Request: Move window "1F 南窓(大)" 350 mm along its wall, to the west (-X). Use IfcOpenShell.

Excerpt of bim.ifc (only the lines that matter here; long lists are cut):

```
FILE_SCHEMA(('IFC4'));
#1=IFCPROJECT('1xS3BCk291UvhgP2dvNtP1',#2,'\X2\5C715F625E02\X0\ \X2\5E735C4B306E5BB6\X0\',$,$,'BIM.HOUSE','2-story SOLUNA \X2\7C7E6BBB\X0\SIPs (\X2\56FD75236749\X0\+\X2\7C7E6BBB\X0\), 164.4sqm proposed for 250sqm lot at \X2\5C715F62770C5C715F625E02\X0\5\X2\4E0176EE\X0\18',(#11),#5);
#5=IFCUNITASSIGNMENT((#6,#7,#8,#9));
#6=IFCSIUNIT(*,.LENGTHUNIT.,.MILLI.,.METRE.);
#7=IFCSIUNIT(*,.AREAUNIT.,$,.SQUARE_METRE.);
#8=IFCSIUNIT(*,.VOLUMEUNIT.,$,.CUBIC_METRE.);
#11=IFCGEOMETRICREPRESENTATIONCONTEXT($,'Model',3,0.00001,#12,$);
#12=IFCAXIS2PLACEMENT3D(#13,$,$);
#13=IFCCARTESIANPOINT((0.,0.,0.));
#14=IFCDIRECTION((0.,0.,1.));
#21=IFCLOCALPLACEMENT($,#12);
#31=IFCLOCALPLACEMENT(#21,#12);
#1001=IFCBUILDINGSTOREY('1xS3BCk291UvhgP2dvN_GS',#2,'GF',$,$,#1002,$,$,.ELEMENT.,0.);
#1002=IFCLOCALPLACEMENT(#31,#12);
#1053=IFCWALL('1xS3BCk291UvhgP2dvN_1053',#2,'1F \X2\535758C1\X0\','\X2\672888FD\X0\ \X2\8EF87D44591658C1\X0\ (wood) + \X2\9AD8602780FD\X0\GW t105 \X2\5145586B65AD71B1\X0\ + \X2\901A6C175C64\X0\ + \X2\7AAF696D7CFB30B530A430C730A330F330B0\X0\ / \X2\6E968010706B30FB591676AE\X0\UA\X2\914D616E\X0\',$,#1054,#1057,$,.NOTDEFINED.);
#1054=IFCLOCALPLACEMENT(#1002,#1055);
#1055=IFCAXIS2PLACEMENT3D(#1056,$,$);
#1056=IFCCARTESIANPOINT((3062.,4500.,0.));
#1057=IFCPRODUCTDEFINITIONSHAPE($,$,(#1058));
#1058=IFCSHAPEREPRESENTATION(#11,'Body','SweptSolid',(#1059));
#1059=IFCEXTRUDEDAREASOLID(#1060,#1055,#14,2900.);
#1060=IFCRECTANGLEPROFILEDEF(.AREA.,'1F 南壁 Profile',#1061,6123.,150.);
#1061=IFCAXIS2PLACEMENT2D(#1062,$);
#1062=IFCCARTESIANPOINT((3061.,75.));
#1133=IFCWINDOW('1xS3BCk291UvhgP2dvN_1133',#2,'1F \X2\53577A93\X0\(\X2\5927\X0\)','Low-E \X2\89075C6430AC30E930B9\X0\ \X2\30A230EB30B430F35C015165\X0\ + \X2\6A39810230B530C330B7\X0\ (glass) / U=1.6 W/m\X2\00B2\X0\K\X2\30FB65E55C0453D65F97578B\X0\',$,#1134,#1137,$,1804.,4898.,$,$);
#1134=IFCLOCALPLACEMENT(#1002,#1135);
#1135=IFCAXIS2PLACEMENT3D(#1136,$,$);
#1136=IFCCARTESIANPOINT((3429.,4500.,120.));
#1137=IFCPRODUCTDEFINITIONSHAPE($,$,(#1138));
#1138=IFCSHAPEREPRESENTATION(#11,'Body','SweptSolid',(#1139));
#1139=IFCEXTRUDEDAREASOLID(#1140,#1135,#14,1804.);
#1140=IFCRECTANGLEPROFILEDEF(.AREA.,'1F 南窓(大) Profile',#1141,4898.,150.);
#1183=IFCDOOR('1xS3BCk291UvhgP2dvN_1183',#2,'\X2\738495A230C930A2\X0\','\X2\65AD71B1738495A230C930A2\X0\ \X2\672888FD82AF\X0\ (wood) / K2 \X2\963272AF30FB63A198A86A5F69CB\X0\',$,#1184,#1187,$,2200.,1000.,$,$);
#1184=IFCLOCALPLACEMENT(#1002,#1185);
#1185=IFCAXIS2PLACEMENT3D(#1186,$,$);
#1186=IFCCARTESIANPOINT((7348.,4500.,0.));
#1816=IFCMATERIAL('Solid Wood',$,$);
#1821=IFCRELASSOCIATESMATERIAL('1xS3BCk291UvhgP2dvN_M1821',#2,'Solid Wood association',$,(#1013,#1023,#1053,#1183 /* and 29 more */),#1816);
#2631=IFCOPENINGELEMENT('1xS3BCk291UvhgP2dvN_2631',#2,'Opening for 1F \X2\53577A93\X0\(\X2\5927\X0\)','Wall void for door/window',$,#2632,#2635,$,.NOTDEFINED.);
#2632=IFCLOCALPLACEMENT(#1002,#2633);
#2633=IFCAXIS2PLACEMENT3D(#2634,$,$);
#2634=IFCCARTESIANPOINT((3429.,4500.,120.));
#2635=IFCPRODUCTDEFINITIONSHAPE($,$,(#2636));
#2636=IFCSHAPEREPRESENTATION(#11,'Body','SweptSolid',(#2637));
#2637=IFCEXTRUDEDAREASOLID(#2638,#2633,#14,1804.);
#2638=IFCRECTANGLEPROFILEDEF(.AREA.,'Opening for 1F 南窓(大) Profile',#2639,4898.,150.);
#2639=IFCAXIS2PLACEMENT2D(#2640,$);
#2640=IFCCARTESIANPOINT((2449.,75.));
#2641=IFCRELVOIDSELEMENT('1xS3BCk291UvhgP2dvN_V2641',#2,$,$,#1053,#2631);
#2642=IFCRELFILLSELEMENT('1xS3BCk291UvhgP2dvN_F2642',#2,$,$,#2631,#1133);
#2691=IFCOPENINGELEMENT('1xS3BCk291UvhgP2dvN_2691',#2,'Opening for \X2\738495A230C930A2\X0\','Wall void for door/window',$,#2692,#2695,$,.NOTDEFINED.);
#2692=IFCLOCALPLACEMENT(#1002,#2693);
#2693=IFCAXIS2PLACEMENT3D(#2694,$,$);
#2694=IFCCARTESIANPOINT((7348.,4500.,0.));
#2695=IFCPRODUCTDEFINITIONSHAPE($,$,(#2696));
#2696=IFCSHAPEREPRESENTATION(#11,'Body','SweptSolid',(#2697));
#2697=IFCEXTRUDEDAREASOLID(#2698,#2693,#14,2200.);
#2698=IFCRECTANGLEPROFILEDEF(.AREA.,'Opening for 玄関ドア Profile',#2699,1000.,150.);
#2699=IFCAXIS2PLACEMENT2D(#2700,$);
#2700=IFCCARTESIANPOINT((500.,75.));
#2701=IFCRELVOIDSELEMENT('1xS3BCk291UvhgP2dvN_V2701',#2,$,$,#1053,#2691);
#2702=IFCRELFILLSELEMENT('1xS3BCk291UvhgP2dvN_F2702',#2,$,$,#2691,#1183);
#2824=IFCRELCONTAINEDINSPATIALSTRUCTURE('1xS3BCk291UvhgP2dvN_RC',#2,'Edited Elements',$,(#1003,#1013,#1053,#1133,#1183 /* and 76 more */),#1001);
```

```python
import ifcopenshell
import ifcopenshell.api.geometry
import ifcopenshell.util.placement
import ifcopenshell.util.unit

model = ifcopenshell.open("bim.ifc")
unit_scale = ifcopenshell.util.unit.calculate_unit_scale(model)

window = model.by_id(1133)
opening = window.FillsVoids[0].RelatingOpeningElement
wall = opening.VoidsElements[0].RelatingBuildingElement

wall_matrix = ifcopenshell.util.placement.get_local_placement(wall.ObjectPlacement)
shift = wall_matrix[:3, 0] * -0.35 / unit_scale
before = ifcopenshell.util.placement.get_local_placement(window.ObjectPlacement)[:3, 3].copy()

# The window is not placed relative to its opening, so move both.
for product in (opening, window):
    matrix = ifcopenshell.util.placement.get_local_placement(product.ObjectPlacement)
    matrix[:3, 3] += shift
    ifcopenshell.api.geometry.edit_object_placement(model, product=product, matrix=matrix, is_si=False)

after = ifcopenshell.util.placement.get_local_placement(window.ObjectPlacement)[:3, 3]
print("window moved by", (after - before).round(3) + 0.0)

model.write("bim_rev.ifc")
```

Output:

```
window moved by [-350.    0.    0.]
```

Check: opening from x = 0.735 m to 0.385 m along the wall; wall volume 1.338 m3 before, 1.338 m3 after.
